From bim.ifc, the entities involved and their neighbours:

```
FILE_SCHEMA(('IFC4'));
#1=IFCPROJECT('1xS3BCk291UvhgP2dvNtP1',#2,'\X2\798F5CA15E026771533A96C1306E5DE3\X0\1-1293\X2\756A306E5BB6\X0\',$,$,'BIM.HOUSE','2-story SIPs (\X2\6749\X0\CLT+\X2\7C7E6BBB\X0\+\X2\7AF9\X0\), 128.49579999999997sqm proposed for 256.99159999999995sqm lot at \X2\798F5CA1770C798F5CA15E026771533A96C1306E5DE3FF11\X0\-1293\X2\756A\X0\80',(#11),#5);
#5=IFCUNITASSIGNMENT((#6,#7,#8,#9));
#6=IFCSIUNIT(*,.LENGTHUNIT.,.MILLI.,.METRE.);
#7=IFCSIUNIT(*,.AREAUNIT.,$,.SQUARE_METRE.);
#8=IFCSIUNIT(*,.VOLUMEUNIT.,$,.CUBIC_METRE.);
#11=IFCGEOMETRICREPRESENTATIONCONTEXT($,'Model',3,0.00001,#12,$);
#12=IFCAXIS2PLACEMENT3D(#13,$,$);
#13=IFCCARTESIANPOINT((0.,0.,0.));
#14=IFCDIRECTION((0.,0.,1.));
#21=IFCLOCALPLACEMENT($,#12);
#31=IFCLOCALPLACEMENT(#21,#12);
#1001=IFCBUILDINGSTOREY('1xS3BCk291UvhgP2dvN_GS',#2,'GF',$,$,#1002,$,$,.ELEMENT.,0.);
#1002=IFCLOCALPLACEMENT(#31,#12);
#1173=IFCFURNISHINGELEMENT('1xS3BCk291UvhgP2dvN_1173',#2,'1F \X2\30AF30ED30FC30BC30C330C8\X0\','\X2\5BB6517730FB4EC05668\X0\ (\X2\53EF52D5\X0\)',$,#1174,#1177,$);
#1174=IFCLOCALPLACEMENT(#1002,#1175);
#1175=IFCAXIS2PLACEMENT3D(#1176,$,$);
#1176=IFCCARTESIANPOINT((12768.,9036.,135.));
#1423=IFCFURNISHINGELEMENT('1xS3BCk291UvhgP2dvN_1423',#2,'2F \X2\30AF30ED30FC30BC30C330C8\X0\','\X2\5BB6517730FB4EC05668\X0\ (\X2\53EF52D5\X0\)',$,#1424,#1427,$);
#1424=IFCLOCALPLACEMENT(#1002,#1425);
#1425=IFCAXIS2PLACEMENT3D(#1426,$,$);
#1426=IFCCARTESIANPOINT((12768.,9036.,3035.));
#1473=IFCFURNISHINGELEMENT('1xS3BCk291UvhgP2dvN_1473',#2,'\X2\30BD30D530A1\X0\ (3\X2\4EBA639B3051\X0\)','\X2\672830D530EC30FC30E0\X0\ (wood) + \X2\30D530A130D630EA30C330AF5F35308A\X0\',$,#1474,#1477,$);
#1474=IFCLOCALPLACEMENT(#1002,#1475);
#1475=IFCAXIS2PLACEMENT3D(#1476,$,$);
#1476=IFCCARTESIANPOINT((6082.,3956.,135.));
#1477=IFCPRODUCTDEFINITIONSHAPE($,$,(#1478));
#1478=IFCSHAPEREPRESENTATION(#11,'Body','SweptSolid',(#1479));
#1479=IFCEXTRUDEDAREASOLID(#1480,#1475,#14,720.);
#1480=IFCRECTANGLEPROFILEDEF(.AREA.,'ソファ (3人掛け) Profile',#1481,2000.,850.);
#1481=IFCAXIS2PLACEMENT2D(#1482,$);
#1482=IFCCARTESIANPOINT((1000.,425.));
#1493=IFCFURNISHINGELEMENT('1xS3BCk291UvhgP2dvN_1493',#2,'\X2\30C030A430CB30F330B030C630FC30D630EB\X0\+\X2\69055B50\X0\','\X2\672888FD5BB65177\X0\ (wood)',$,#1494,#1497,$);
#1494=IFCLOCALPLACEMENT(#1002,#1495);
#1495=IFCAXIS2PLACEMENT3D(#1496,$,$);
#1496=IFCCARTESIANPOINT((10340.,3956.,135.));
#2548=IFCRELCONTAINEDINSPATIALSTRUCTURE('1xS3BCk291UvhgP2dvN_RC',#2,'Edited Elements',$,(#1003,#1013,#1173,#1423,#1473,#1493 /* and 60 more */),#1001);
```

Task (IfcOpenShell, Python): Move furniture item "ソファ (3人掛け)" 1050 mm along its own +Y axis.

```python
import ifcopenshell
import ifcopenshell.api.geometry
import ifcopenshell.util.placement
import ifcopenshell.util.unit

model = ifcopenshell.open("bim.ifc")
unit_scale = ifcopenshell.util.unit.calculate_unit_scale(model)

item = model.by_id(1473)
matrix = ifcopenshell.util.placement.get_local_placement(item.ObjectPlacement)
matrix[:3, 3] += matrix[:3, 1] * 1.05 / unit_scale
ifcopenshell.api.geometry.edit_object_placement(model, product=item, matrix=matrix, is_si=False)

print(ifcopenshell.util.placement.get_local_placement(item.ObjectPlacement).round(3) + 0.0)

model.write("bim_edited.ifc")
```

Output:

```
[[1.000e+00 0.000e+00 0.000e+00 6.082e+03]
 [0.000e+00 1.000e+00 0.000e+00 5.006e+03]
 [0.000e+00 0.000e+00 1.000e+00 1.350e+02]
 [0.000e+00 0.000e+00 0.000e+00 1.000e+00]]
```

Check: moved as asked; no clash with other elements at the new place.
